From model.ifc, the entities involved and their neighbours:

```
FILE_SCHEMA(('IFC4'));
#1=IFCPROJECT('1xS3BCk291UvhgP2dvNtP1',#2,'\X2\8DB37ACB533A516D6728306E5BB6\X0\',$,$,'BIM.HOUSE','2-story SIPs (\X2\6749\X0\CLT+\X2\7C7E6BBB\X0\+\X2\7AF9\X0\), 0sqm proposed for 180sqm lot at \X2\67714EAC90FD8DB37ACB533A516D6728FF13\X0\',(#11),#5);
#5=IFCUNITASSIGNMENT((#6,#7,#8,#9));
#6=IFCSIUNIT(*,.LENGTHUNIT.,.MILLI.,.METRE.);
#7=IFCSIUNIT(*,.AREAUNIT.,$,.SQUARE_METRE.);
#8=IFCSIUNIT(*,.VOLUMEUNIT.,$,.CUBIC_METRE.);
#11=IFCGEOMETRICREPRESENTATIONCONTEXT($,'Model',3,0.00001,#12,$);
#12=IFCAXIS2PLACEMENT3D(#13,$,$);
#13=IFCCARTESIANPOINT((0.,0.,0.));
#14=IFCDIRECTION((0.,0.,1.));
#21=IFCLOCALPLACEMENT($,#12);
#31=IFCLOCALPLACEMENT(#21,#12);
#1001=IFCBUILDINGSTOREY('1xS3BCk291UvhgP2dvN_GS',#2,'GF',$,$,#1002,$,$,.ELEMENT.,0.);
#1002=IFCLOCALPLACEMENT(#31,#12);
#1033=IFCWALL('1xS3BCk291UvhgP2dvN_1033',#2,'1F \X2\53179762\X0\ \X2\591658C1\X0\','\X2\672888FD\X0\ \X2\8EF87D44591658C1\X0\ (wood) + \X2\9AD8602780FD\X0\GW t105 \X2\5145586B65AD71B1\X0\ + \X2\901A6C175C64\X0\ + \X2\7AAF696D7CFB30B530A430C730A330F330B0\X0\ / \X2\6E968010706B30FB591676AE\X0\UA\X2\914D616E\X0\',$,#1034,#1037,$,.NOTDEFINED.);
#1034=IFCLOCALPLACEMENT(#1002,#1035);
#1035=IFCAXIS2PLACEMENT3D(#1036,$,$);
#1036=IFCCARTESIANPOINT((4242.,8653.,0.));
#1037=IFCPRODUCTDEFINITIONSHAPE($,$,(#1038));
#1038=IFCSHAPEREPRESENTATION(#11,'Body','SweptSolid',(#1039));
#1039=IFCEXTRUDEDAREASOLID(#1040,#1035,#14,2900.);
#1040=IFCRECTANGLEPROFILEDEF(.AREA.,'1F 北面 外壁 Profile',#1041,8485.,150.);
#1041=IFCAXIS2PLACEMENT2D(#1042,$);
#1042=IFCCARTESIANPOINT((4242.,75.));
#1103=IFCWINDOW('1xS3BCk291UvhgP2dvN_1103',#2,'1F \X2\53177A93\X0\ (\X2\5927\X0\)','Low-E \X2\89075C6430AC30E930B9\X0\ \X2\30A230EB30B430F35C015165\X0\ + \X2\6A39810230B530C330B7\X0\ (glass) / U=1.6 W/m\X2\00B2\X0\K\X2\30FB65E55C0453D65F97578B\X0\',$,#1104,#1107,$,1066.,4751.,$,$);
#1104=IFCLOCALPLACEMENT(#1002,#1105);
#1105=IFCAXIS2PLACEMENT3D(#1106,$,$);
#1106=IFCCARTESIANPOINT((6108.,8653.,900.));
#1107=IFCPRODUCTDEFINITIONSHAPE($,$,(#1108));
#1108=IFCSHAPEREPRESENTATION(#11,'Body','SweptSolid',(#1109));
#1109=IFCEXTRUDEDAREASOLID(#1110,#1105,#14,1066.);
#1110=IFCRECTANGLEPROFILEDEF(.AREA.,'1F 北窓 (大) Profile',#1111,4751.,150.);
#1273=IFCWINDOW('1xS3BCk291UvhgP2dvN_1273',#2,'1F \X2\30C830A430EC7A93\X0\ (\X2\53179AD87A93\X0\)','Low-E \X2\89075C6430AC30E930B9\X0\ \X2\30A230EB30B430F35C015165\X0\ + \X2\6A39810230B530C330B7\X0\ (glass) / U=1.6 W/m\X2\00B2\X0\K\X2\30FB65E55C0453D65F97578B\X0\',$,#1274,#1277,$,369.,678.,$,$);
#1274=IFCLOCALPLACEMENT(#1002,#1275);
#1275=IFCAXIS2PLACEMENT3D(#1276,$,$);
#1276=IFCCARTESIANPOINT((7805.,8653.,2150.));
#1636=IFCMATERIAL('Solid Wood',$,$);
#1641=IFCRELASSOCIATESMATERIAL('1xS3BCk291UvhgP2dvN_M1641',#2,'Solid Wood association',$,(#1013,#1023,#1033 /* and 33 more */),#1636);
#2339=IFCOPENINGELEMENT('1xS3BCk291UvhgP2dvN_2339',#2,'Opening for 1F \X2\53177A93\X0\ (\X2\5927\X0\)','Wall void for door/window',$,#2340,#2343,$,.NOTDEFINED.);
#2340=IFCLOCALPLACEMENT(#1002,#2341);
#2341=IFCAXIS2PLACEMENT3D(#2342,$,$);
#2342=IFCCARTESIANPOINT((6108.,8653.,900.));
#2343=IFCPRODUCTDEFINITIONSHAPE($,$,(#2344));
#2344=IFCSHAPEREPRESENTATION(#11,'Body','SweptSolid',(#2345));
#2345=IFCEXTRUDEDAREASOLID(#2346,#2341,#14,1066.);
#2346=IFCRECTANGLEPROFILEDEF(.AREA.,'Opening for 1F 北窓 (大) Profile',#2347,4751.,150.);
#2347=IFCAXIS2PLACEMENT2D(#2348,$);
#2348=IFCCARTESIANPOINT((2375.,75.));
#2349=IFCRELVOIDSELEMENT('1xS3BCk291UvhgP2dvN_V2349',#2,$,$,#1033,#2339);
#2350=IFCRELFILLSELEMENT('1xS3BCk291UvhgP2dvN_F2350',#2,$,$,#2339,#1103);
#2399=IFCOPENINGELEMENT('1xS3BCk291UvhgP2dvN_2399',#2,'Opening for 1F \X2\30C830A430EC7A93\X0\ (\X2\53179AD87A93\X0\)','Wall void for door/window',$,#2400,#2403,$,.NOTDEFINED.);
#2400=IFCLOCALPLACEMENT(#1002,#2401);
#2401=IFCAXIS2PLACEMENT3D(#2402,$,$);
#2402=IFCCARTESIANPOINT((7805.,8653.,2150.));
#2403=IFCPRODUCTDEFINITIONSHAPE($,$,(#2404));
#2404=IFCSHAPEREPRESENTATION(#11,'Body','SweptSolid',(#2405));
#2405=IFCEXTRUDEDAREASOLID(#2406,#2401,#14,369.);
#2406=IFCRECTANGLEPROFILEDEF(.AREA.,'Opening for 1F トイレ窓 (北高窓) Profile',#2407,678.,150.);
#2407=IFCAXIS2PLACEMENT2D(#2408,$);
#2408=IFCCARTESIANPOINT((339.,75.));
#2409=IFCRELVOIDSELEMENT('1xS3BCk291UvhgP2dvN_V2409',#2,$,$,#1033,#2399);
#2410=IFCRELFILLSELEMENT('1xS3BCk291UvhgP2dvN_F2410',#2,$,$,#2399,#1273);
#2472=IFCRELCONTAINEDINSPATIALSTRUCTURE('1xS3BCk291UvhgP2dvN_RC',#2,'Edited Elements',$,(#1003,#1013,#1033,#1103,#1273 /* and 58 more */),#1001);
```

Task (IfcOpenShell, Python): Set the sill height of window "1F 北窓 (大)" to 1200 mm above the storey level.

```python
import numpy as np
import ifcopenshell
import ifcopenshell.api.geometry
import ifcopenshell.geom
import ifcopenshell.util.element
import ifcopenshell.util.placement
import ifcopenshell.util.shape
import ifcopenshell.util.unit

model = ifcopenshell.open("model.ifc")
unit_scale = ifcopenshell.util.unit.calculate_unit_scale(model)

window = model.by_guid("1xS3BCk291UvhgP2dvN_1103")
opening = window.FillsVoids[0].RelatingOpeningElement
storey = ifcopenshell.util.element.get_container(window, ifc_class="IfcBuildingStorey")
level = ifcopenshell.util.placement.get_local_placement(storey.ObjectPlacement)[2, 3]

# The opening's origin need not be at the sill, so measure its lowest point.
shape = ifcopenshell.geom.create_shape(ifcopenshell.geom.settings(), opening)
bottom = ifcopenshell.util.shape.get_shape_bottom_elevation(shape, shape.geometry) / unit_scale
dz = level + 1200.0 - bottom

shift = np.array([0.0, 0.0, dz])
# The window is not placed relative to its opening, so move both.
for product in (opening, window):
    matrix = ifcopenshell.util.placement.get_local_placement(product.ObjectPlacement)
    matrix[:3, 3] += shift
    ifcopenshell.api.geometry.edit_object_placement(model, product=product, matrix=matrix, is_si=False)

print(f"moved by {dz * unit_scale:+.3f} m")

model.write("model_edited.ifc")
```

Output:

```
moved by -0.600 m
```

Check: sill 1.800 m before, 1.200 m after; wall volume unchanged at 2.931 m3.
